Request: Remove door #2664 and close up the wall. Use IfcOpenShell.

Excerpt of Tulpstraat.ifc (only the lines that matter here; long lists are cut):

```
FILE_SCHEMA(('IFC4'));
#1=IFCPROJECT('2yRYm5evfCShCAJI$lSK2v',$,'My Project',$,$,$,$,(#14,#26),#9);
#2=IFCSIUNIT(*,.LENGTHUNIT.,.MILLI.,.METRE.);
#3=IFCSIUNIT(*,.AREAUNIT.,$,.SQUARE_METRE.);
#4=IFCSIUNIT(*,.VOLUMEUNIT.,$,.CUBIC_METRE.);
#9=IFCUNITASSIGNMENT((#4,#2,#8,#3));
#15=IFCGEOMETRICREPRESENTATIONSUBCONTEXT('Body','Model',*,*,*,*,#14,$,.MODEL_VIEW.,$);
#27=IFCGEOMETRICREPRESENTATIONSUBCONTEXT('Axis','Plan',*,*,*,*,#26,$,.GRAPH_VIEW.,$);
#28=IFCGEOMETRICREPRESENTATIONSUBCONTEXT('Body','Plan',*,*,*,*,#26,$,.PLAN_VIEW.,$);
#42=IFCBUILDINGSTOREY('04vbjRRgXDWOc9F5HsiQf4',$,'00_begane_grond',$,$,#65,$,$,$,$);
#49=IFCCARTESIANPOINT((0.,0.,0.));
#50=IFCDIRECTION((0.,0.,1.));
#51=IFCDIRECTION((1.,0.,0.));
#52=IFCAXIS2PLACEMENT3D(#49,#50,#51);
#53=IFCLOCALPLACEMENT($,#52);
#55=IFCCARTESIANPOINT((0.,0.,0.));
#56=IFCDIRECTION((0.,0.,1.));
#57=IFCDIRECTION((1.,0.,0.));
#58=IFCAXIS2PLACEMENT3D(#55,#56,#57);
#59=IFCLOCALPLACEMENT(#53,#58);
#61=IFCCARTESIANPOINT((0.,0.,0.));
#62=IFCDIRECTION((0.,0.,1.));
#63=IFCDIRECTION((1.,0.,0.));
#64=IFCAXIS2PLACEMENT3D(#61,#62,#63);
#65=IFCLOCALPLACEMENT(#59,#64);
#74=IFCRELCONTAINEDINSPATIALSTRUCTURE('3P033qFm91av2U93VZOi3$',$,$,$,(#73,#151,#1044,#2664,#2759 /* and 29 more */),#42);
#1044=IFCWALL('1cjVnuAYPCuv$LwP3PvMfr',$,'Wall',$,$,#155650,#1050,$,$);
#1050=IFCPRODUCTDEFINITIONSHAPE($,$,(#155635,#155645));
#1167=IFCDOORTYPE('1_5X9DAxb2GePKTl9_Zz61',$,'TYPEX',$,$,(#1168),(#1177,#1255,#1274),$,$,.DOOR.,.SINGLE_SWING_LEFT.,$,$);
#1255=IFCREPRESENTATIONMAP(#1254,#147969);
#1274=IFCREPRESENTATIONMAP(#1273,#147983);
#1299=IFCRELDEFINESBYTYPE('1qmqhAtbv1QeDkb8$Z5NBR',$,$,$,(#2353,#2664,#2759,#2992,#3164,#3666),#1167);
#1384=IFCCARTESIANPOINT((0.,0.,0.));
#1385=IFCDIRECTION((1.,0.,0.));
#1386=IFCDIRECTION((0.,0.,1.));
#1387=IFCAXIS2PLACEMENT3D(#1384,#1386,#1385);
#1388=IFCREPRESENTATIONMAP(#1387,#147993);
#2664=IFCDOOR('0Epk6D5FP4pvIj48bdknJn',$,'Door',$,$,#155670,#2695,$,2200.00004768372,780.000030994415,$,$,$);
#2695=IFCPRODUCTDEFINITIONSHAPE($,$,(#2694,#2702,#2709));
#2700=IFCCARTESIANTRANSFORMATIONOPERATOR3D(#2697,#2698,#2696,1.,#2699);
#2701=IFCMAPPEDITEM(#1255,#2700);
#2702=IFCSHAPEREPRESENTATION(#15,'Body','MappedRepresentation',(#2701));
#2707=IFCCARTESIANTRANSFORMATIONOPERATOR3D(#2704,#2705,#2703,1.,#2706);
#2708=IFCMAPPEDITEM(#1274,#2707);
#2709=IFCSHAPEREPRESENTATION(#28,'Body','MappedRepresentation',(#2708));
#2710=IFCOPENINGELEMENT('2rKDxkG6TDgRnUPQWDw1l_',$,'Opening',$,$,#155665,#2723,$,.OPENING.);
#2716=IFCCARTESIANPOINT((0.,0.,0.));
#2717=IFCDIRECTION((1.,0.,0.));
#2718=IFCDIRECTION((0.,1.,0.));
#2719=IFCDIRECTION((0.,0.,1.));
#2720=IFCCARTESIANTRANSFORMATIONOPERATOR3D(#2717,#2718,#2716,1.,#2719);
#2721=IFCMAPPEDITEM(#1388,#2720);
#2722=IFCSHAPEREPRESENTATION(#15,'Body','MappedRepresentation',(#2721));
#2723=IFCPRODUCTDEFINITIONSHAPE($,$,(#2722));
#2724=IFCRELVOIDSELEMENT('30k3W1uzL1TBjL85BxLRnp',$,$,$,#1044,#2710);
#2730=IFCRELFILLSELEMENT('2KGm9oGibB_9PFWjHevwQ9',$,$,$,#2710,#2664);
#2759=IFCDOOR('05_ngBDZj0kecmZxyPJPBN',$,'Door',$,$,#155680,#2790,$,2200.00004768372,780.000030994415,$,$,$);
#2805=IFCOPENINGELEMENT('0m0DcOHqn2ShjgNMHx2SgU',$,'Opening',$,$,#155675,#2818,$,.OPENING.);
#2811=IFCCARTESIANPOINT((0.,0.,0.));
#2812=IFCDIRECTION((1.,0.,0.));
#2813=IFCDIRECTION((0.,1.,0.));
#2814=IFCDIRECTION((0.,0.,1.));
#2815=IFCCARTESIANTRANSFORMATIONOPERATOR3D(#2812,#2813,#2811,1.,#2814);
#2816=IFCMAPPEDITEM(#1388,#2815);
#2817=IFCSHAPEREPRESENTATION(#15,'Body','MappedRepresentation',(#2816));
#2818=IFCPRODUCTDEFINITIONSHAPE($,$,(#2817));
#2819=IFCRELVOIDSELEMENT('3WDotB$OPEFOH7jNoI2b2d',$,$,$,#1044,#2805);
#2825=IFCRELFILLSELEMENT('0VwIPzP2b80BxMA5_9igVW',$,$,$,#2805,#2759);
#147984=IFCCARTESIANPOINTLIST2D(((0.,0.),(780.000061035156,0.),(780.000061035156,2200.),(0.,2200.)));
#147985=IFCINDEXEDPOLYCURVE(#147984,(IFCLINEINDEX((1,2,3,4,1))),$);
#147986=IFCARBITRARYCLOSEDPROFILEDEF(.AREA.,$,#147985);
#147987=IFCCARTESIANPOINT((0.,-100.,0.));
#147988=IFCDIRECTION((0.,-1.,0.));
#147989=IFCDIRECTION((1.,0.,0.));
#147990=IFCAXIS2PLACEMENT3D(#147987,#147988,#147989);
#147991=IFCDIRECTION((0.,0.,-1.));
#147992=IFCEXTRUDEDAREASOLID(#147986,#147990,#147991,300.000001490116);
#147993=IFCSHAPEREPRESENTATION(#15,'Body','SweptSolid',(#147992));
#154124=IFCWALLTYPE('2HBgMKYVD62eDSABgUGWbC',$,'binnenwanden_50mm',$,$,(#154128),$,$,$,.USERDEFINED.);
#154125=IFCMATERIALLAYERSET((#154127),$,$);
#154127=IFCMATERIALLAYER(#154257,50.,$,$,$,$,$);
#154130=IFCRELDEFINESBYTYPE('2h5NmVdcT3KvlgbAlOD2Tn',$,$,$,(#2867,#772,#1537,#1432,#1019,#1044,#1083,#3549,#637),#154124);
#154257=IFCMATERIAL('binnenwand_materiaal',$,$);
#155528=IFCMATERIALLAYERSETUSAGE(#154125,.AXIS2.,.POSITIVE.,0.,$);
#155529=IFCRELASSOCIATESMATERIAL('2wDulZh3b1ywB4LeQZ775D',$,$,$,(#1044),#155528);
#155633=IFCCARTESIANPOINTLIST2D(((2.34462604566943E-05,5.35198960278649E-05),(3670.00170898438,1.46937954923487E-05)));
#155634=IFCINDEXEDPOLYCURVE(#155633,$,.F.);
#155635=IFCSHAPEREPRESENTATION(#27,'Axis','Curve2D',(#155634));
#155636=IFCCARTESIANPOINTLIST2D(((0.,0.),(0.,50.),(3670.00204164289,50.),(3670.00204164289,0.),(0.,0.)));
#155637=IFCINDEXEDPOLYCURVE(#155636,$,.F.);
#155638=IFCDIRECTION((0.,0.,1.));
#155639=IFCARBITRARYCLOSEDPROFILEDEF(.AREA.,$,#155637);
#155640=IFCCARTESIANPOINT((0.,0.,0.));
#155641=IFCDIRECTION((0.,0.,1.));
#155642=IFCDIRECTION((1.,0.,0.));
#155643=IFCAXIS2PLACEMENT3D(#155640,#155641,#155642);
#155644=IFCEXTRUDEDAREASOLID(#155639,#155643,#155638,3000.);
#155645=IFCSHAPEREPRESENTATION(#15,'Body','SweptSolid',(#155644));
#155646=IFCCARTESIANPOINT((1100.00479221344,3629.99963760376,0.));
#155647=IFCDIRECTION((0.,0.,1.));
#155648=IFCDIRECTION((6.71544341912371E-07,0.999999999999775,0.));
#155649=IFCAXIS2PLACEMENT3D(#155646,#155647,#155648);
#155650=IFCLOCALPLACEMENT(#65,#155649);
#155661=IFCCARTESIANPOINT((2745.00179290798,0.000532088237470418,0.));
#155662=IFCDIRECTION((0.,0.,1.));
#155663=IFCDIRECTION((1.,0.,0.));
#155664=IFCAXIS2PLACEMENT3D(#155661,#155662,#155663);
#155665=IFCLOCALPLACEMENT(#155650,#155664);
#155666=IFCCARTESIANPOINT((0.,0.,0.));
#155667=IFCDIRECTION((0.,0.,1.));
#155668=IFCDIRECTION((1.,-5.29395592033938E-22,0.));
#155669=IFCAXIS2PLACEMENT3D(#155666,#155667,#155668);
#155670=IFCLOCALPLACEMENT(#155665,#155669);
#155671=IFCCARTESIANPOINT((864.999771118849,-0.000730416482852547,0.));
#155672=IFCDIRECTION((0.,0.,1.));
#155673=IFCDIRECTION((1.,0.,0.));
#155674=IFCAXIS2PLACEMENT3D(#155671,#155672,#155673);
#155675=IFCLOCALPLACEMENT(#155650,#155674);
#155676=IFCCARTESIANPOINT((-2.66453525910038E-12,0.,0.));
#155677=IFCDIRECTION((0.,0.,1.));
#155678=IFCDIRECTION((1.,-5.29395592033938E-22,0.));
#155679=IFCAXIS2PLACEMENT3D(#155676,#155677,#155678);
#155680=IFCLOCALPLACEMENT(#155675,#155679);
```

```python
import ifcopenshell
import ifcopenshell.api.feature
import ifcopenshell.api.root
import ifcopenshell.geom
import ifcopenshell.util.shape

model = ifcopenshell.open("Tulpstraat.ifc")
settings = ifcopenshell.geom.settings()


def volume(element):
    """Net volume in cubic metres, openings subtracted."""
    shape = ifcopenshell.geom.create_shape(settings, element)
    return ifcopenshell.util.shape.get_volume(shape.geometry)


door = model.by_id(2664)
opening = door.FillsVoids[0].RelatingOpeningElement
wall = opening.VoidsElements[0].RelatingBuildingElement
before = volume(wall)

ifcopenshell.api.root.remove_product(model, product=door)
ifcopenshell.api.feature.remove_feature(model, feature=opening)

after = volume(wall)

print(f"wall volume {before:.3f} -> {after:.3f} m3")

model.write("Tulpstraat-out.ifc")
```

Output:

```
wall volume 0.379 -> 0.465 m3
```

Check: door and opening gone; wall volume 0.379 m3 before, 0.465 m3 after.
